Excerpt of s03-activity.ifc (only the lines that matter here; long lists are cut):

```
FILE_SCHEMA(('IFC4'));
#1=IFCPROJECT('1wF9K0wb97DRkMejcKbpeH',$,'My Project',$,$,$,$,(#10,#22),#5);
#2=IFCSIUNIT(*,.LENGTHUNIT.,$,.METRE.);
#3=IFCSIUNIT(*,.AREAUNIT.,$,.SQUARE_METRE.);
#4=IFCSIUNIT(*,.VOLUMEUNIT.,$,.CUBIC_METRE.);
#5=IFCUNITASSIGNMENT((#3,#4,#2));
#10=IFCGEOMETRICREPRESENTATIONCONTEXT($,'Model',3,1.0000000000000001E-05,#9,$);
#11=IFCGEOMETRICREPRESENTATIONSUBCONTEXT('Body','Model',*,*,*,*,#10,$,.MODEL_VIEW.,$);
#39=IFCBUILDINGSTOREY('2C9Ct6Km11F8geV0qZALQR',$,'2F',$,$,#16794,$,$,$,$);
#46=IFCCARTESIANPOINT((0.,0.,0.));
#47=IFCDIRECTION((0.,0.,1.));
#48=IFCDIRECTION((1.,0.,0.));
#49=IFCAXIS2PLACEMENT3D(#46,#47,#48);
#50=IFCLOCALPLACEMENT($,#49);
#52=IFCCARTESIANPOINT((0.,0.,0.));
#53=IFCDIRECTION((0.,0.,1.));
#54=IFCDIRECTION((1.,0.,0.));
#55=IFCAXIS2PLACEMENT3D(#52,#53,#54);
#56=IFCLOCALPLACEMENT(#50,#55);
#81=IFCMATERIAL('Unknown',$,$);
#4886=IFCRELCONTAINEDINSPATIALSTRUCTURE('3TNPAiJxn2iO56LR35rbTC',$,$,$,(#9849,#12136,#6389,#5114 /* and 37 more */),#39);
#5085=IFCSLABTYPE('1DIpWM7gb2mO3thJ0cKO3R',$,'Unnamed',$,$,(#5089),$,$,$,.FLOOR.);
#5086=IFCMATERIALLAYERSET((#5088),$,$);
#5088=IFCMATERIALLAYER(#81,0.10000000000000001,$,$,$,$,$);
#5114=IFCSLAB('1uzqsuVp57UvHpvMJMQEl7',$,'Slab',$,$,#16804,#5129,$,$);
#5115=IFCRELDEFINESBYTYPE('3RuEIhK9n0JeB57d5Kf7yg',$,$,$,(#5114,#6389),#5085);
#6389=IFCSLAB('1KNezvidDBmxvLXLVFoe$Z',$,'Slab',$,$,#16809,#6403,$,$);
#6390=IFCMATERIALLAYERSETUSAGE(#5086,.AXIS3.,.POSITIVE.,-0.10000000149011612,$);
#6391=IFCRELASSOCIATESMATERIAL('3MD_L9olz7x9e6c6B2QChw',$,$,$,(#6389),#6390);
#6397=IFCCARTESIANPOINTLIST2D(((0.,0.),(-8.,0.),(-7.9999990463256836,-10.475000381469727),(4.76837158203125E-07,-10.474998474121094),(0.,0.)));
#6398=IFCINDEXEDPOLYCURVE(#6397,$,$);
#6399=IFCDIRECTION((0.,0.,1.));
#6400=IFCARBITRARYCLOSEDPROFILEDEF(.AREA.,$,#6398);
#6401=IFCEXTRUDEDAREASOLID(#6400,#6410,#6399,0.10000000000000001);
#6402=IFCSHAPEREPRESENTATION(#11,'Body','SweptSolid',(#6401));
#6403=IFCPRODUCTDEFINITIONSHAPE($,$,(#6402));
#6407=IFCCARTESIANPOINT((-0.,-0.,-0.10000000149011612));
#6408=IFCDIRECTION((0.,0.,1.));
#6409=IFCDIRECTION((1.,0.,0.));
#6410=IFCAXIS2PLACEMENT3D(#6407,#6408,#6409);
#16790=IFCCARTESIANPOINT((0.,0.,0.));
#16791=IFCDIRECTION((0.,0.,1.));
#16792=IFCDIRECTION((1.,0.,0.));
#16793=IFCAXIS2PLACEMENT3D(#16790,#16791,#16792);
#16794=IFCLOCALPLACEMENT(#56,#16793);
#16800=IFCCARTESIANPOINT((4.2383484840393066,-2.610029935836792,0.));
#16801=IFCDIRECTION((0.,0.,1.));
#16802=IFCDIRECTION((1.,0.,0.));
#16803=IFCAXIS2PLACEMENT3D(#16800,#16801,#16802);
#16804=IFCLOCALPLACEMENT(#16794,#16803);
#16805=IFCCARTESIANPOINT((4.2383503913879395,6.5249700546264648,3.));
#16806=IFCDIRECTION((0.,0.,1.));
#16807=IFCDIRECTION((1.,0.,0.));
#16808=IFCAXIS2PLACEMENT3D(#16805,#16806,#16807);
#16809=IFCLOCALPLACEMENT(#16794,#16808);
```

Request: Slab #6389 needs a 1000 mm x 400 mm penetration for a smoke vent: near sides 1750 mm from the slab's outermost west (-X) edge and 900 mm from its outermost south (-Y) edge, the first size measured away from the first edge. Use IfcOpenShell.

```python
import numpy as np
import ifcopenshell
import ifcopenshell.api.feature
import ifcopenshell.api.geometry
import ifcopenshell.api.root
import ifcopenshell.geom
import ifcopenshell.util.placement
import ifcopenshell.util.representation
import ifcopenshell.util.shape
import ifcopenshell.util.unit

model = ifcopenshell.open("s03-activity.ifc")
unit_scale = ifcopenshell.util.unit.calculate_unit_scale(model)
settings = ifcopenshell.geom.settings()


def volume(element):
    """Net volume in cubic metres, openings subtracted."""
    shape = ifcopenshell.geom.create_shape(settings, element)
    return ifcopenshell.util.shape.get_volume(shape.geometry)


slab = model.by_guid("1KNezvidDBmxvLXLVFoe$Z")
before = volume(slab)

# Extent in the slab's own axes, in metres. The edges named are its -X and -Y sides.
slab_shape = ifcopenshell.geom.create_shape(settings, slab)
vertices = ifcopenshell.util.shape.get_vertices(slab_shape.geometry)
x_min, y_min, bottom = vertices.min(axis=0)
top = vertices[:, 2].max()

opening = ifcopenshell.api.root.create_entity(model, ifc_class="IfcOpeningElement", name="Smoke vent opening", predefined_type="OPENING")
context = ifcopenshell.util.representation.get_context(model, "Model", "Body", "MODEL_VIEW")
width, depth = 1, 0.4
outline = [(0.0, 0.0), (width, 0.0), (width, depth), (0.0, depth), (0.0, 0.0)]
# Overshoot both faces by 50 mm so the cut is clean.
shape = ifcopenshell.api.geometry.add_slab_representation(
    model, context=context, depth=top - bottom + 0.1, polyline=outline
)
ifcopenshell.api.geometry.assign_representation(model, product=opening, representation=shape)

matrix = ifcopenshell.util.placement.get_local_placement(slab.ObjectPlacement)
matrix[:, 3] = matrix @ np.append(np.array([x_min + 1.75, y_min + 0.9, bottom - 0.05]) / unit_scale, 1.0)
ifcopenshell.api.geometry.edit_object_placement(model, product=opening, matrix=matrix, is_si=False)
ifcopenshell.api.feature.add_feature(model, feature=opening, element=slab)

after = volume(slab)

print(f"slab volume {before:.3f} -> {after:.3f} m3")

model.write("s03-activity_updated.ifc")
```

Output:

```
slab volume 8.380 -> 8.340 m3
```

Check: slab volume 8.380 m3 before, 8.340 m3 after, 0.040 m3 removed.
